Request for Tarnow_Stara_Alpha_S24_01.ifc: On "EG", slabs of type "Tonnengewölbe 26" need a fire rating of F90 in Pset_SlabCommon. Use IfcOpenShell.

First a look at what the model holds.

```python
import ifcopenshell
import ifcopenshell.util.element

model = ifcopenshell.open("Tarnow_Stara_Alpha_S24_01.ifc")
print(model.schema)
storey = next(s for s in model.by_type("IfcBuildingStorey") if s.Name == "EG")
slabs = [e for e in ifcopenshell.util.element.get_decomposition(storey) if e.is_a("IfcSlab")]
seen = {}
for e in slabs:
    element_type = ifcopenshell.util.element.get_type(e)
    key = (element_type.Name if element_type != e and element_type else None, ifcopenshell.util.element.get_pset(e, "Pset_SlabCommon", "FireRating"))
    seen[key] = seen.get(key, 0) + 1
for (name, value), count in sorted(seen.items(), key=str):
    print(count, "x", name, "|", value)
```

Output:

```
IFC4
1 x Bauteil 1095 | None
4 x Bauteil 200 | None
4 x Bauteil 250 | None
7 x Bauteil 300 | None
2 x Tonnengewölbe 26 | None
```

```python
import ifcopenshell
import ifcopenshell.api.pset
import ifcopenshell.util.element

model = ifcopenshell.open("Tarnow_Stara_Alpha_S24_01.ifc")

storey = next(s for s in model.by_type("IfcBuildingStorey") if s.Name == "EG")
slabs = [e for e in ifcopenshell.util.element.get_decomposition(storey) if e.is_a("IfcSlab")]

count = 0
for e in slabs:
    element_type = ifcopenshell.util.element.get_type(e)
    if element_type in (None, e) or element_type.Name != "Tonnengewölbe 26":
        continue
    # add_pset returns the element's existing set when there is one.
    pset = ifcopenshell.api.pset.add_pset(model, product=e, name="Pset_SlabCommon")
    ifcopenshell.api.pset.edit_pset(model, pset=pset, properties={"FireRating": "F90"})
    count += 1

print(count, "slabs updated")

model.write("Tarnow_Stara_Alpha_S24_01_rev.ifc")
```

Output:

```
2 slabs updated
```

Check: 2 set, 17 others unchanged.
